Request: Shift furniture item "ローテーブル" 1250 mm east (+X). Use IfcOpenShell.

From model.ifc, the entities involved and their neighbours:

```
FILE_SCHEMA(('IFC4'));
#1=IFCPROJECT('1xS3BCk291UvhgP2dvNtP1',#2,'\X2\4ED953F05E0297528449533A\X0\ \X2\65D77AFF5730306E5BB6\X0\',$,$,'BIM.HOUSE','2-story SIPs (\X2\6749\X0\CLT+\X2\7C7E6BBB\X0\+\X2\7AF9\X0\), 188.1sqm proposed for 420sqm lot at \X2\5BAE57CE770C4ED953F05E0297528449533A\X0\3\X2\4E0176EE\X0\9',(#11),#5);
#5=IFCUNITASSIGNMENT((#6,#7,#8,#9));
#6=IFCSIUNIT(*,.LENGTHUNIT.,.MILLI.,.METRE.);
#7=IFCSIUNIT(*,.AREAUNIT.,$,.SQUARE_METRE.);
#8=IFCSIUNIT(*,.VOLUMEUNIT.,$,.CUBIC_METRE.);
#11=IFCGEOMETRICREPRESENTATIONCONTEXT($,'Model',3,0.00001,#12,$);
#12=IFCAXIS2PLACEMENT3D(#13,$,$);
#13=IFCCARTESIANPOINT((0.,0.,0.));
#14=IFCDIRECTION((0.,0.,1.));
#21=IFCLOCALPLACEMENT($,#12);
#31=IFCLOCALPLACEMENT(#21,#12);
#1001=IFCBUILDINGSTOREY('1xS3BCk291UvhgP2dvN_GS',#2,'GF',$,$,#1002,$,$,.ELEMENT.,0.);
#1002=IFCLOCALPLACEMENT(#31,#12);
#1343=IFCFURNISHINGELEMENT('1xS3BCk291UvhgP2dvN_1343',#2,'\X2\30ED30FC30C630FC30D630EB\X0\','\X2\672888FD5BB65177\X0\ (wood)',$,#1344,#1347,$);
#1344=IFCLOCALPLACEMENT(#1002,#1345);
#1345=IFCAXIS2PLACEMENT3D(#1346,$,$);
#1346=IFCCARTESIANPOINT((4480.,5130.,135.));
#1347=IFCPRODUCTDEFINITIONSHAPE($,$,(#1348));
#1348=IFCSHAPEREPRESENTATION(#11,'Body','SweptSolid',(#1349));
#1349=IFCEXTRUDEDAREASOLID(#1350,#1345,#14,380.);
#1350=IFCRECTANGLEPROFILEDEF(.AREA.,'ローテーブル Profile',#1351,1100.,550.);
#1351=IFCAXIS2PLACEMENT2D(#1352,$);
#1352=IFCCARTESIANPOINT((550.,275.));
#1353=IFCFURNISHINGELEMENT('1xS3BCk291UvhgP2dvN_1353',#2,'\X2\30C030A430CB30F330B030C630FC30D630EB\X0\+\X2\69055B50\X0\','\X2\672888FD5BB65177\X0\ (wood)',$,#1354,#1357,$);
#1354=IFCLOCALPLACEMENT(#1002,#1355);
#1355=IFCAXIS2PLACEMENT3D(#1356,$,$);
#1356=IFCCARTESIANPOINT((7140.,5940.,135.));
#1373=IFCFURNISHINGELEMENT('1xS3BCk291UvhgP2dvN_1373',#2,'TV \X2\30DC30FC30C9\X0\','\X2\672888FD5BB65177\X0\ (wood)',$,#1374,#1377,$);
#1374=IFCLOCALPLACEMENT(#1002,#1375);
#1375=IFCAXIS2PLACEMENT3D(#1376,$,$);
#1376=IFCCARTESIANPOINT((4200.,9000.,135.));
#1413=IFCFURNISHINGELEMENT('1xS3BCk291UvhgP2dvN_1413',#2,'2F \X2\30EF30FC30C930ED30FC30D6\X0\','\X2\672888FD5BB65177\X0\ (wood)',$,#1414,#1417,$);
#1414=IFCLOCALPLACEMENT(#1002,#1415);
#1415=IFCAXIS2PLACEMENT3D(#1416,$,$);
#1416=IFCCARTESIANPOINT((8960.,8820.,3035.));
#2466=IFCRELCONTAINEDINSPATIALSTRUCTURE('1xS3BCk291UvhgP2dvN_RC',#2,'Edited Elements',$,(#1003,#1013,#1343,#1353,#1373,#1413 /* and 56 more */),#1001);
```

```python
import ifcopenshell
import ifcopenshell.api.geometry
import ifcopenshell.util.placement
import ifcopenshell.util.unit

model = ifcopenshell.open("model.ifc")
unit_scale = ifcopenshell.util.unit.calculate_unit_scale(model)

item = model.by_guid("1xS3BCk291UvhgP2dvN_1343")
matrix = ifcopenshell.util.placement.get_local_placement(item.ObjectPlacement)
matrix[0, 3] += 1.25 / unit_scale
ifcopenshell.api.geometry.edit_object_placement(model, product=item, matrix=matrix, is_si=False)

print(ifcopenshell.util.placement.get_local_placement(item.ObjectPlacement).round(3) + 0.0)

model.write("model_updated.ifc")
```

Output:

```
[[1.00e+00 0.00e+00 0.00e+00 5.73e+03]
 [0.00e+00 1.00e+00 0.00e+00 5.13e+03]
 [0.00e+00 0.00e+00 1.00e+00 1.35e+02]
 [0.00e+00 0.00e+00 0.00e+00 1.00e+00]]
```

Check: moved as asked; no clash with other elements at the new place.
